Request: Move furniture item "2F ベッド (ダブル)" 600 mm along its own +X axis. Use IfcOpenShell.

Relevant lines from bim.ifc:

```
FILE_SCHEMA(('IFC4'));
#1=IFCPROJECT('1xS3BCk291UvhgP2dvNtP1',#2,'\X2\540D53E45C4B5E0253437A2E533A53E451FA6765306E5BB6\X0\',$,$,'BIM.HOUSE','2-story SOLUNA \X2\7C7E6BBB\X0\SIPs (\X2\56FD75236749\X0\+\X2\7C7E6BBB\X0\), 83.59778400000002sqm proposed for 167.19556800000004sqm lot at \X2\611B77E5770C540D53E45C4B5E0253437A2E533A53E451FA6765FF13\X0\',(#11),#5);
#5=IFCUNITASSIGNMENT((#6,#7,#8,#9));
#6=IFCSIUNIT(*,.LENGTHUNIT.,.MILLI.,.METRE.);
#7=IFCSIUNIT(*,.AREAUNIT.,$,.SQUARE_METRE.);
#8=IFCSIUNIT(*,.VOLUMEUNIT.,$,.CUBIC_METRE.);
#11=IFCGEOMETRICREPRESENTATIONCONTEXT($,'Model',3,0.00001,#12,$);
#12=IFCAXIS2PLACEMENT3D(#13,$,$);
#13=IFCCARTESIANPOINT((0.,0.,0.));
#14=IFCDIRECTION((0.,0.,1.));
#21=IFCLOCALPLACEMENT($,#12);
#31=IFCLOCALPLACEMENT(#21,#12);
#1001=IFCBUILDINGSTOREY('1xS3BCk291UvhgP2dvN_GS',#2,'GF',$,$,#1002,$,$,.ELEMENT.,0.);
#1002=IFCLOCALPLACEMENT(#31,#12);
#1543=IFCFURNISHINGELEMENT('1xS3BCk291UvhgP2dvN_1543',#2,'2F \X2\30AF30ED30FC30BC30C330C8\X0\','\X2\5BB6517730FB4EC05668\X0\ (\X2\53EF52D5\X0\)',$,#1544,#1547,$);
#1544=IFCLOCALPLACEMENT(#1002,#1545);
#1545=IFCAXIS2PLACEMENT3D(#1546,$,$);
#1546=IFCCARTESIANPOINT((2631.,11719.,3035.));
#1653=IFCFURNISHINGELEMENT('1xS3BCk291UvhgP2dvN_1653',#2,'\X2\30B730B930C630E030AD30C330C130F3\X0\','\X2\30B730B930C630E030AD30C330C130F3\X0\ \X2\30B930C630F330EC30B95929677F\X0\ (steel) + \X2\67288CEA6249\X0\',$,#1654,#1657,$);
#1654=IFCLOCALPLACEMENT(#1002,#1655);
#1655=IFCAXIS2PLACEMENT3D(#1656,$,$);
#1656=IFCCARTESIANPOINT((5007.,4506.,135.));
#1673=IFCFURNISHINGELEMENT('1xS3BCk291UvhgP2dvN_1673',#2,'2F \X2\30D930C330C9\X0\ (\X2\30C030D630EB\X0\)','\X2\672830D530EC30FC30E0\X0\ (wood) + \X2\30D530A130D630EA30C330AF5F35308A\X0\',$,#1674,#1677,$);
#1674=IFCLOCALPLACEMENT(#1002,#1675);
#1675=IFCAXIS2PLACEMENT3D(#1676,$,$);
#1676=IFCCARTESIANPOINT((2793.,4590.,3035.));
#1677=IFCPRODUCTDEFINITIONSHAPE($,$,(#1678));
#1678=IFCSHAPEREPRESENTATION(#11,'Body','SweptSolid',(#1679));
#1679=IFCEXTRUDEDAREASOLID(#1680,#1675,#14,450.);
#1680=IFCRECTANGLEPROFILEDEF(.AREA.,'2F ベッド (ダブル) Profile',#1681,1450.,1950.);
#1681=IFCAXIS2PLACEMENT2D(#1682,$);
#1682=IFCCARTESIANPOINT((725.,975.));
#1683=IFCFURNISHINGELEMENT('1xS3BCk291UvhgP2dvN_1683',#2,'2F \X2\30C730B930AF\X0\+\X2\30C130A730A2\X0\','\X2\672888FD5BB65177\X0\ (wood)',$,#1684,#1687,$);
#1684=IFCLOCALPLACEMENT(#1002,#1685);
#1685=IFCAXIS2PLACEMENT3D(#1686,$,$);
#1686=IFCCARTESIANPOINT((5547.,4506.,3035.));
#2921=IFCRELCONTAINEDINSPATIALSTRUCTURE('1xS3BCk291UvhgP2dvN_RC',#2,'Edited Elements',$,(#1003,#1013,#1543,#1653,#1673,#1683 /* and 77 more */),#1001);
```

```python
import ifcopenshell
import ifcopenshell.api.geometry
import ifcopenshell.util.placement

model = ifcopenshell.open("bim.ifc")

item = model.by_guid("1xS3BCk291UvhgP2dvN_1673")
matrix = ifcopenshell.util.placement.get_local_placement(item.ObjectPlacement)
matrix[:3, 3] += matrix[:3, 0] * 600.0
ifcopenshell.api.geometry.edit_object_placement(model, product=item, matrix=matrix, is_si=False)

print(ifcopenshell.util.placement.get_local_placement(item.ObjectPlacement).round(3) + 0.0)

model.write("bim_updated.ifc")
```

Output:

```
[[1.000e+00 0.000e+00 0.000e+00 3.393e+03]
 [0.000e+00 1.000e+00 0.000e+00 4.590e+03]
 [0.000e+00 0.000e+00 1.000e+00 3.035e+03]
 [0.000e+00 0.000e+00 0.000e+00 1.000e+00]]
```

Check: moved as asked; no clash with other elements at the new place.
